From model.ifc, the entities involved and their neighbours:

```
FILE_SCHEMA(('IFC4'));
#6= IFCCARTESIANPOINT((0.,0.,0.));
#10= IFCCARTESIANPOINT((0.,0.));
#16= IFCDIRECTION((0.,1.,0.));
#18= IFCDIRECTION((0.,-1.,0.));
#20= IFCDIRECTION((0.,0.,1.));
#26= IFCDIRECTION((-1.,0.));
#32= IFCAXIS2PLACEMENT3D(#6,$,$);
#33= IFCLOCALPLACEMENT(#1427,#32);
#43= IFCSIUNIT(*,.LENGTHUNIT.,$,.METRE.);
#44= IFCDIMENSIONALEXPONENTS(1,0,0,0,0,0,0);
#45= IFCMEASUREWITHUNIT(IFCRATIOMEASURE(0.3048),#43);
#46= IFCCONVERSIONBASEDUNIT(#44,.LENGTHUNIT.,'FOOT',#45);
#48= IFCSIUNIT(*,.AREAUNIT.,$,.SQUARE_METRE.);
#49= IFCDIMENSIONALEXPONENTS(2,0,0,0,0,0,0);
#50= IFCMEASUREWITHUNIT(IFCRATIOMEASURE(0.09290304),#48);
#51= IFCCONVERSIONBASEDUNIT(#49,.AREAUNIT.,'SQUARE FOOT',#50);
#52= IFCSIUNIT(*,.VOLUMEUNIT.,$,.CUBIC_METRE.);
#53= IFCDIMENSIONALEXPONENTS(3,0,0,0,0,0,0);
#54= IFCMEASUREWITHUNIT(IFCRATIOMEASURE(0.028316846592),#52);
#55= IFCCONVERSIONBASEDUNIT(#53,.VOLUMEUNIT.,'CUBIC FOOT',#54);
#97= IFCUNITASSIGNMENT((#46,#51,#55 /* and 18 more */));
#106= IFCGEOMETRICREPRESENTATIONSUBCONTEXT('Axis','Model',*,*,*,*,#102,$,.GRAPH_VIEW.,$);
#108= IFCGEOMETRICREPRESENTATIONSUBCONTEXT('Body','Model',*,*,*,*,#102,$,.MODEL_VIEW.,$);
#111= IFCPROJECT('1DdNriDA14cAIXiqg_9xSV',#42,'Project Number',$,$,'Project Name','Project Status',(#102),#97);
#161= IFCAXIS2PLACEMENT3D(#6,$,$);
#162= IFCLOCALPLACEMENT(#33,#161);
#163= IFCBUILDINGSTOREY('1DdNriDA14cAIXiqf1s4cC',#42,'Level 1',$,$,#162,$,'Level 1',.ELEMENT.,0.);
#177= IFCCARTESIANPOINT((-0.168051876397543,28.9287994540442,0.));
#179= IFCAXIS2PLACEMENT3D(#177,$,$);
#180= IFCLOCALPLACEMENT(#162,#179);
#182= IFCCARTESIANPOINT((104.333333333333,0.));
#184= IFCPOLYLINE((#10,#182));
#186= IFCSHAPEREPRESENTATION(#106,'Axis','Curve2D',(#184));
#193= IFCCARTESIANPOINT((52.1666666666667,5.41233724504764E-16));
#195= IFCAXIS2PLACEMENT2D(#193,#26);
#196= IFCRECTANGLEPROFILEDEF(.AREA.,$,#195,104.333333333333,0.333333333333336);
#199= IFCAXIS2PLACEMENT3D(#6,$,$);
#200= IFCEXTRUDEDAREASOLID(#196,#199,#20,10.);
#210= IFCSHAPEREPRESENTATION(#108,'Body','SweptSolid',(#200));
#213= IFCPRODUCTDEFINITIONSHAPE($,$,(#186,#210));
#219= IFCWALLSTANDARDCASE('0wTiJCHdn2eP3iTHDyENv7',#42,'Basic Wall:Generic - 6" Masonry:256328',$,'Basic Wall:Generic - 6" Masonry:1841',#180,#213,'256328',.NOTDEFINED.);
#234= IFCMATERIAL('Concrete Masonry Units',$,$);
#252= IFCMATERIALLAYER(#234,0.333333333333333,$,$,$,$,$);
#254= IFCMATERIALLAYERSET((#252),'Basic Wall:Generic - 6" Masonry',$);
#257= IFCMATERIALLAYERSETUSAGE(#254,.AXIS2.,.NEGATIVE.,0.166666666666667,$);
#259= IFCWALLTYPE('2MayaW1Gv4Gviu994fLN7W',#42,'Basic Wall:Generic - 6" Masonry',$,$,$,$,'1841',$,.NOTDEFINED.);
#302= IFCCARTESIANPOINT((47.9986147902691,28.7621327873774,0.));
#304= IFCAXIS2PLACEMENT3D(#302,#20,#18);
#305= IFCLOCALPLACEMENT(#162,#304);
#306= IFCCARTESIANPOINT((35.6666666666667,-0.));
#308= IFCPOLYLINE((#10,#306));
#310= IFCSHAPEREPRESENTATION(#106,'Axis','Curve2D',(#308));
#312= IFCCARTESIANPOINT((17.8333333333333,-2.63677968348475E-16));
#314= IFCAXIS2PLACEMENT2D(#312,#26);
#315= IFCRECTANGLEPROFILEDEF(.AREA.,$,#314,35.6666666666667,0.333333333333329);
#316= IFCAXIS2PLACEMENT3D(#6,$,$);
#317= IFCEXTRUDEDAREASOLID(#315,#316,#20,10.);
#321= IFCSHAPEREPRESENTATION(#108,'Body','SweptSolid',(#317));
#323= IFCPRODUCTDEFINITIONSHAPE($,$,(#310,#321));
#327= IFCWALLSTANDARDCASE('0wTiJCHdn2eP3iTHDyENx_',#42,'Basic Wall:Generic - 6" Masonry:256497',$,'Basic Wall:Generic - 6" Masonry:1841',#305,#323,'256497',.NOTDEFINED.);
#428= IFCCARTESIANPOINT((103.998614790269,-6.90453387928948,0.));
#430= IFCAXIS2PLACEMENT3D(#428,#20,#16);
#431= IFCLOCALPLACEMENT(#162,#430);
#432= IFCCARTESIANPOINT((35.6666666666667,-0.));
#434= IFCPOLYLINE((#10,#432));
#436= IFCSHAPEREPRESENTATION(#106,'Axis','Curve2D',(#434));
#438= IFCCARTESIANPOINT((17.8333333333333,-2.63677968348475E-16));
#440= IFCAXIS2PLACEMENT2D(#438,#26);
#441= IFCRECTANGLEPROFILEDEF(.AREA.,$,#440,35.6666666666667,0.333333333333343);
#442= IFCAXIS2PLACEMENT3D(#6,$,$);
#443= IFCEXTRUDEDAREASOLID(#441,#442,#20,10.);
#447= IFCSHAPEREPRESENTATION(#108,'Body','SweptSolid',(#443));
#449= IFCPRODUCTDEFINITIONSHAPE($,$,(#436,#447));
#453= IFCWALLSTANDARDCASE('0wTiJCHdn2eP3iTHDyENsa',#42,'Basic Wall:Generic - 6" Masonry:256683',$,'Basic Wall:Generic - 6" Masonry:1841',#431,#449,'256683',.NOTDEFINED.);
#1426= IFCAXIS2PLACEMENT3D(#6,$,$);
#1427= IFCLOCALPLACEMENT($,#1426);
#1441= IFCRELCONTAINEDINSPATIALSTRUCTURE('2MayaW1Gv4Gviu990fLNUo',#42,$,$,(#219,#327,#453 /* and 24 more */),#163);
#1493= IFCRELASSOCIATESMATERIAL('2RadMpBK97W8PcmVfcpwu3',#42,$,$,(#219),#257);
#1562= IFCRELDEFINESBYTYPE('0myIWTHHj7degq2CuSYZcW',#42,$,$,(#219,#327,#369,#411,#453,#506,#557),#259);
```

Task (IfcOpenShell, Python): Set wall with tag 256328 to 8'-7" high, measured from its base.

```python
import ifcopenshell
import ifcopenshell.geom
import ifcopenshell.util.representation
import ifcopenshell.util.shape
import ifcopenshell.util.unit

model = ifcopenshell.open("model.ifc")
unit_scale = ifcopenshell.util.unit.calculate_unit_scale(model)
settings = ifcopenshell.geom.settings()


def volume(element):
    """Net volume in cubic metres, openings subtracted."""
    shape = ifcopenshell.geom.create_shape(settings, element)
    return ifcopenshell.util.shape.get_volume(shape.geometry)


wall = model.by_guid("0wTiJCHdn2eP3iTHDyENv7")
before = volume(wall)

body = ifcopenshell.util.representation.get_representation(wall, "Model", "Body")
solid = body.Items[0]
old_height = solid.Depth
solid.Depth = 103 * 0.0254 / unit_scale
after = volume(wall)

print(f"height {old_height:g} -> {solid.Depth:g}, volume {before:.3f} -> {after:.3f} m3")

model.write("model_rev.ifc")
```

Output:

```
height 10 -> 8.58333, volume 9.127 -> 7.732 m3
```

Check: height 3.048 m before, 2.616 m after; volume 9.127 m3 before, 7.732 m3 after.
